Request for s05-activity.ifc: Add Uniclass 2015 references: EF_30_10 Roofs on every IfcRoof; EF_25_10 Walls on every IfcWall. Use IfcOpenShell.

First a look at what the model holds.

```python
import ifcopenshell

model = ifcopenshell.open("s05-activity.ifc")
print(model.schema)
print("classifications:", [c.Name for c in model.by_type("IfcClassification")])
for ifc_class in ("IfcDoor", "IfcRoof", "IfcStair", "IfcWall", "IfcWindow"):
    print(ifc_class, len(model.by_type(ifc_class)))
```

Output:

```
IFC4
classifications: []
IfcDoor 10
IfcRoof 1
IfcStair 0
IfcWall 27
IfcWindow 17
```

```python
import ifcopenshell
import ifcopenshell.api.classification

model = ifcopenshell.open("s05-activity.ifc")

system = ifcopenshell.api.classification.add_classification(model, classification="Uniclass 2015")

codes = {
    "IfcRoof": ("EF_30_10", "Roofs"),
    "IfcWall": ("EF_25_10", "Walls"),
}
for ifc_class, (code, name) in codes.items():
    products = model.by_type(ifc_class)
    ifcopenshell.api.classification.add_reference(
        model, products=products, classification=system, identification=code, name=name
    )
    print(code, len(products))

model.write("s05-activity_rev.ifc")
```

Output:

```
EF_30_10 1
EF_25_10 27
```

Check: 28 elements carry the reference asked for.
